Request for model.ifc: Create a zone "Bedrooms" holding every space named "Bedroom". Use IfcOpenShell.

First a look at what the model holds.

```python
import ifcopenshell

model = ifcopenshell.open("model.ifc")
print(model.schema)
seen = {}
for space in model.by_type("IfcSpace"):
    seen[space.LongName] = seen.get(space.LongName, 0) + 1
for name, count in sorted(seen.items(), key=str):
    print(count, "x", name)
print("zones:", [z.Name for z in model.by_type("IfcZone")][:20])
```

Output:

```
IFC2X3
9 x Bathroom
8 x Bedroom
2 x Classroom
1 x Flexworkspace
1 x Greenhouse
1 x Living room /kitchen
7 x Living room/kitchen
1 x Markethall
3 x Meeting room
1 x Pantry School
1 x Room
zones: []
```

```python
import ifcopenshell
import ifcopenshell.api.group
import ifcopenshell.api.root

model = ifcopenshell.open("model.ifc")

names = {"Bedroom"}
spaces = [s for s in model.by_type("IfcSpace") if s.LongName in names]

zone = ifcopenshell.api.root.create_entity(model, ifc_class="IfcZone", name="Bedrooms")
ifcopenshell.api.group.assign_group(model, products=spaces, group=zone)
print(len(spaces), "spaces in", zone.Name)

model.write("model_rev.ifc")
```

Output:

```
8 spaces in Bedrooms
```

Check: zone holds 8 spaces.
